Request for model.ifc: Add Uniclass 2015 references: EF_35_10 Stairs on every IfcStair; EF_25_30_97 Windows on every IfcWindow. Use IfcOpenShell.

First a look at what the model holds.

```python
import ifcopenshell

model = ifcopenshell.open("model.ifc")
print(model.schema)
print("classifications:", [c.Name for c in model.by_type("IfcClassification")])
for ifc_class in ("IfcDoor", "IfcRoof", "IfcStair", "IfcWall", "IfcWindow"):
    print(ifc_class, len(model.by_type(ifc_class)))
```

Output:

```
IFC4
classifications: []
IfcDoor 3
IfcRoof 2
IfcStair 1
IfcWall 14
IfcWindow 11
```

```python
import ifcopenshell
import ifcopenshell.api.classification

model = ifcopenshell.open("model.ifc")

system = ifcopenshell.api.classification.add_classification(model, classification="Uniclass 2015")

codes = {
    "IfcStair": ("EF_35_10", "Stairs"),
    "IfcWindow": ("EF_25_30_97", "Windows"),
}
for ifc_class, (code, name) in codes.items():
    products = model.by_type(ifc_class)
    ifcopenshell.api.classification.add_reference(
        model, products=products, classification=system, identification=code, name=name
    )
    print(code, len(products))

model.write("model-out.ifc")
```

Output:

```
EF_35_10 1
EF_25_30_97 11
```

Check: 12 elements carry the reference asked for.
